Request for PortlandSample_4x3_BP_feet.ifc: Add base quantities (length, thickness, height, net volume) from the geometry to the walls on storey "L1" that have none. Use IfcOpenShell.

First a look at what the model holds.

```python
import ifcopenshell
import ifcopenshell.util.element
import ifcopenshell.util.unit

model = ifcopenshell.open("PortlandSample_4x3_BP_feet.ifc")
print(model.schema)
for unit_type in ("LENGTHUNIT", "AREAUNIT", "VOLUMEUNIT"):
    print(unit_type, ifcopenshell.util.unit.calculate_unit_scale(model, unit_type))
storey = next(s for s in model.by_type("IfcBuildingStorey") if s.Name == "L1")
walls = [e for e in ifcopenshell.util.element.get_decomposition(storey) if e.is_a("IfcWall")]
for e in sorted(walls, key=lambda e: e.id()):
    print(e.id(), e.is_a(), e.Name, list(ifcopenshell.util.element.get_psets(e, qtos_only=True)), sep=" | ")
```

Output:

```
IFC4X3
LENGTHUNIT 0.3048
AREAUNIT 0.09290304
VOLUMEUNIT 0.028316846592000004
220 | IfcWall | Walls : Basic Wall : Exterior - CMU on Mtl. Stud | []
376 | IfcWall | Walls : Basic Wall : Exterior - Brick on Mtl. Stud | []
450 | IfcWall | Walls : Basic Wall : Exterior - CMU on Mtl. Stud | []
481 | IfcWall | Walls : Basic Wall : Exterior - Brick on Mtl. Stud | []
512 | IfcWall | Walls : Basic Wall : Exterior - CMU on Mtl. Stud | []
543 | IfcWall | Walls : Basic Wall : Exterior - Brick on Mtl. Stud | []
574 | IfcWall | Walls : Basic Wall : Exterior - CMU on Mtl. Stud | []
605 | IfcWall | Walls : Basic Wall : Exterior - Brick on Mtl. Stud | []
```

```python
import ifcopenshell
import ifcopenshell.api.pset
import ifcopenshell.geom
import ifcopenshell.util.element
import ifcopenshell.util.shape
import ifcopenshell.util.unit

model = ifcopenshell.open("PortlandSample_4x3_BP_feet.ifc")
unit_scale = ifcopenshell.util.unit.calculate_unit_scale(model)
volume_scale = ifcopenshell.util.unit.calculate_unit_scale(model, "VOLUMEUNIT")
settings = ifcopenshell.geom.settings()

storey = next(s for s in model.by_type("IfcBuildingStorey") if s.Name == "L1")
walls = [e for e in ifcopenshell.util.element.get_decomposition(storey) if e.is_a("IfcWall")]

for e in sorted(walls, key=lambda e: e.id()):
    if ifcopenshell.util.element.get_psets(e, qtos_only=True, should_inherit=False):
        continue
    # Geometry comes back in metres, in the element's own axes.
    shape = ifcopenshell.geom.create_shape(settings, e)
    values = {
        "Length": ifcopenshell.util.shape.get_x(shape.geometry) / unit_scale,
        "Width": ifcopenshell.util.shape.get_y(shape.geometry) / unit_scale,
        "Height": ifcopenshell.util.shape.get_z(shape.geometry) / unit_scale,
        "NetVolume": ifcopenshell.util.shape.get_volume(shape.geometry) / volume_scale,
    }
    qto = ifcopenshell.api.pset.add_qto(model, product=e, name="Qto_WallBaseQuantities")
    ifcopenshell.api.pset.edit_qto(model, qto=qto, properties=values)
    print(e.id(), {k: round(v, 3) for k, v in values.items()})

model.write("PortlandSample_4x3_BP_feet_updated.ifc")
```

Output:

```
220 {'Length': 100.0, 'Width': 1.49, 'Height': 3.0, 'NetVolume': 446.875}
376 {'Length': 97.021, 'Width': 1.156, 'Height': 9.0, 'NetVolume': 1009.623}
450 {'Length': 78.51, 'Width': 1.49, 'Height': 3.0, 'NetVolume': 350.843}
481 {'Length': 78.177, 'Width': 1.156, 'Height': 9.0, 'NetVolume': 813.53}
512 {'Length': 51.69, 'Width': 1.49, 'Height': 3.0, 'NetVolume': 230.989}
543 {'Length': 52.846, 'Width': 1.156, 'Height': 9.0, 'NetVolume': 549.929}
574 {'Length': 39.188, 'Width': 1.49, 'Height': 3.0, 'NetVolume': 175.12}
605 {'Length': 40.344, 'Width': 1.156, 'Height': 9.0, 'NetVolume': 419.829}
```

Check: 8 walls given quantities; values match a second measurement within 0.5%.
